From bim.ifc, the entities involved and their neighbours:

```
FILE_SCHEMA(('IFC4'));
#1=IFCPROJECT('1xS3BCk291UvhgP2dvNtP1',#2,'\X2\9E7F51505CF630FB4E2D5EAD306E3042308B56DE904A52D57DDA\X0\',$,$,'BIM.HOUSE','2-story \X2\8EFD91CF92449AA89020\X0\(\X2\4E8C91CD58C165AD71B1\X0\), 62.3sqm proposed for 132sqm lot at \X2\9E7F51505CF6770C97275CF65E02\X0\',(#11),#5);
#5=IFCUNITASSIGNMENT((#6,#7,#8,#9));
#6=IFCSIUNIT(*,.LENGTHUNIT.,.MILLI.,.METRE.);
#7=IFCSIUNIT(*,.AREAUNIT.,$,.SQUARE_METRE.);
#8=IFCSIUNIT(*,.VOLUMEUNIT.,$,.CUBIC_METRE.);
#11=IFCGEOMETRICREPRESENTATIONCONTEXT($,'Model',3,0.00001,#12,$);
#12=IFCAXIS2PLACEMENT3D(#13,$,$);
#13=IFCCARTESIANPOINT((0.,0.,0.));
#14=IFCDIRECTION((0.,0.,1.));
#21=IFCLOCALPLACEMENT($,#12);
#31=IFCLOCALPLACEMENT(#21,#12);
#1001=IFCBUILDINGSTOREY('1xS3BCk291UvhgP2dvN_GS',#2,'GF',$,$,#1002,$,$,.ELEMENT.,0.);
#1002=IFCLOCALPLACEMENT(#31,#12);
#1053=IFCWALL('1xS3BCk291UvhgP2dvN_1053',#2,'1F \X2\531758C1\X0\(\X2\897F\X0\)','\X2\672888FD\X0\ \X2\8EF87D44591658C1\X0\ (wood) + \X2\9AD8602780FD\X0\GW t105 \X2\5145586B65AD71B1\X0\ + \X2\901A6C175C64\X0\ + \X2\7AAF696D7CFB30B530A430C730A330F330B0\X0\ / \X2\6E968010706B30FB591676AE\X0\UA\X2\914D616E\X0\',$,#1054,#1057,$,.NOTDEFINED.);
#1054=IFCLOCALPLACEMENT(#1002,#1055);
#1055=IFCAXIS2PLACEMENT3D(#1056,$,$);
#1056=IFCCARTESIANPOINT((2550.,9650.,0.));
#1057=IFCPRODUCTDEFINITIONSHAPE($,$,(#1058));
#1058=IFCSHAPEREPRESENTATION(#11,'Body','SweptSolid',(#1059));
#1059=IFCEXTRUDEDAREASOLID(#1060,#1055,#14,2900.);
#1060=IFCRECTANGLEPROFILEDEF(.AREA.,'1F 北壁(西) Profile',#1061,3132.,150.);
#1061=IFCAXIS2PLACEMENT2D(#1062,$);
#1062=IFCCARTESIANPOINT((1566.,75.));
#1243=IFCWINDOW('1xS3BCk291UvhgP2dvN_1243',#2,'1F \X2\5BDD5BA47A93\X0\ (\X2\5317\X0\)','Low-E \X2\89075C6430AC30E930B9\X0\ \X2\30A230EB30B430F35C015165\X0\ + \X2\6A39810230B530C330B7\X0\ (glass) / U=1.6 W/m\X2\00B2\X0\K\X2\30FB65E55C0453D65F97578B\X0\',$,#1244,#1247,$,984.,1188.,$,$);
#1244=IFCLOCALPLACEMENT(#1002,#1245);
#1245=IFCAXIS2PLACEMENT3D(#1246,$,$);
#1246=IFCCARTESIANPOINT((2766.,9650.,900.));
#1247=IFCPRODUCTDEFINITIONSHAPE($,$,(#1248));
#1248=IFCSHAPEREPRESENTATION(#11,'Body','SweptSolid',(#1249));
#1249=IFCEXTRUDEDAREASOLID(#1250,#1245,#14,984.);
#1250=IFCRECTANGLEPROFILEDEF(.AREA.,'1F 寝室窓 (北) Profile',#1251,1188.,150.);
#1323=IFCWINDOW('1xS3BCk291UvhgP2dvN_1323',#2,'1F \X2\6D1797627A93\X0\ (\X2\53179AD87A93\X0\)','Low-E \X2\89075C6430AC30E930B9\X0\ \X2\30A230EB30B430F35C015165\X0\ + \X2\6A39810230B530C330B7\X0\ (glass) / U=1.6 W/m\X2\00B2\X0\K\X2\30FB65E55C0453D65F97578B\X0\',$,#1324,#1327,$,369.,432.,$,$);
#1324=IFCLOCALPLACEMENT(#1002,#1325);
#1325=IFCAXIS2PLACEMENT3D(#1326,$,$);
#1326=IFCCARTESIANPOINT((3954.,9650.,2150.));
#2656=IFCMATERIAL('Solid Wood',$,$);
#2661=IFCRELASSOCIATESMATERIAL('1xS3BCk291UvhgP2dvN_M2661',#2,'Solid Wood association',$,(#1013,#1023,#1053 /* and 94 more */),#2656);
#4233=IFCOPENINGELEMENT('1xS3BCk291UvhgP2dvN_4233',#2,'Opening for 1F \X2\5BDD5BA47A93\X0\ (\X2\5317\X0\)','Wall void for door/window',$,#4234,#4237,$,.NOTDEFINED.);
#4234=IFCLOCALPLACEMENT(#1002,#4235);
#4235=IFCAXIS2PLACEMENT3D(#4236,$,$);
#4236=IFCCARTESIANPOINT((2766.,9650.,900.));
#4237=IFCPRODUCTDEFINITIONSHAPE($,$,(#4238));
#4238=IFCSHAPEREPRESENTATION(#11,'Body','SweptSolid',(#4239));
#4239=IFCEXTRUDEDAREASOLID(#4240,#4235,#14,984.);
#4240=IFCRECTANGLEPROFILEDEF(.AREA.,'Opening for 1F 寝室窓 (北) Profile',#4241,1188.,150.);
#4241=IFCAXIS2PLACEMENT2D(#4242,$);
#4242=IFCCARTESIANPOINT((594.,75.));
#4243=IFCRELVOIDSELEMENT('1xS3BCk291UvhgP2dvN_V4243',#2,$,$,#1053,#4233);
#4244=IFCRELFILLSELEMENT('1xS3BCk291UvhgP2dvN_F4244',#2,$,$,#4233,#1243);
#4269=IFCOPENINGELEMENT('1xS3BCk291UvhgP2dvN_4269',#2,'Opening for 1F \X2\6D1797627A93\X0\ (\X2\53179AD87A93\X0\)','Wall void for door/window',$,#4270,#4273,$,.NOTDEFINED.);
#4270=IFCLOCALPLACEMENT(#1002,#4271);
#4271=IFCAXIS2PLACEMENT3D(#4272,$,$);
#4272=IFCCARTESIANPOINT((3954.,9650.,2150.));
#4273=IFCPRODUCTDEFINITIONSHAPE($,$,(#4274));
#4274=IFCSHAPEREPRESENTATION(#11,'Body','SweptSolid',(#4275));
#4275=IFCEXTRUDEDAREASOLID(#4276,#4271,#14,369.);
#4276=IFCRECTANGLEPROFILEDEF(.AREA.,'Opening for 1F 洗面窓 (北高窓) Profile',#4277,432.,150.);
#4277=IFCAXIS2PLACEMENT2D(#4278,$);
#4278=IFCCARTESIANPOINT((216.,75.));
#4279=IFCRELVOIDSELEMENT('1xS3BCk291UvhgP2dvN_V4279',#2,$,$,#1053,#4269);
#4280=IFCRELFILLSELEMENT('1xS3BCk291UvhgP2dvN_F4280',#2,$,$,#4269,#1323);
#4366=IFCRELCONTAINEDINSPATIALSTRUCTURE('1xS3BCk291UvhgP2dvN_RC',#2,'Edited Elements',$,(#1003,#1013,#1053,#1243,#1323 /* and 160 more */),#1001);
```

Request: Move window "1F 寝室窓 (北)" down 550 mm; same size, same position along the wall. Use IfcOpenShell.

```python
import numpy as np
import ifcopenshell
import ifcopenshell.api.geometry
import ifcopenshell.util.placement
import ifcopenshell.util.unit

model = ifcopenshell.open("bim.ifc")
unit_scale = ifcopenshell.util.unit.calculate_unit_scale(model)

window = model.by_guid("1xS3BCk291UvhgP2dvN_1243")
opening = window.FillsVoids[0].RelatingOpeningElement
dz = -550.0

shift = np.array([0.0, 0.0, dz])
# The window is not placed relative to its opening, so move both.
for product in (opening, window):
    matrix = ifcopenshell.util.placement.get_local_placement(product.ObjectPlacement)
    matrix[:3, 3] += shift
    ifcopenshell.api.geometry.edit_object_placement(model, product=product, matrix=matrix, is_si=False)

print(f"moved by {dz * unit_scale:+.3f} m")

model.write("bim-out.ifc")
```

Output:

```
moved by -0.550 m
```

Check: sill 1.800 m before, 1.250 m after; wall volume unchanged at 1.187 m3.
